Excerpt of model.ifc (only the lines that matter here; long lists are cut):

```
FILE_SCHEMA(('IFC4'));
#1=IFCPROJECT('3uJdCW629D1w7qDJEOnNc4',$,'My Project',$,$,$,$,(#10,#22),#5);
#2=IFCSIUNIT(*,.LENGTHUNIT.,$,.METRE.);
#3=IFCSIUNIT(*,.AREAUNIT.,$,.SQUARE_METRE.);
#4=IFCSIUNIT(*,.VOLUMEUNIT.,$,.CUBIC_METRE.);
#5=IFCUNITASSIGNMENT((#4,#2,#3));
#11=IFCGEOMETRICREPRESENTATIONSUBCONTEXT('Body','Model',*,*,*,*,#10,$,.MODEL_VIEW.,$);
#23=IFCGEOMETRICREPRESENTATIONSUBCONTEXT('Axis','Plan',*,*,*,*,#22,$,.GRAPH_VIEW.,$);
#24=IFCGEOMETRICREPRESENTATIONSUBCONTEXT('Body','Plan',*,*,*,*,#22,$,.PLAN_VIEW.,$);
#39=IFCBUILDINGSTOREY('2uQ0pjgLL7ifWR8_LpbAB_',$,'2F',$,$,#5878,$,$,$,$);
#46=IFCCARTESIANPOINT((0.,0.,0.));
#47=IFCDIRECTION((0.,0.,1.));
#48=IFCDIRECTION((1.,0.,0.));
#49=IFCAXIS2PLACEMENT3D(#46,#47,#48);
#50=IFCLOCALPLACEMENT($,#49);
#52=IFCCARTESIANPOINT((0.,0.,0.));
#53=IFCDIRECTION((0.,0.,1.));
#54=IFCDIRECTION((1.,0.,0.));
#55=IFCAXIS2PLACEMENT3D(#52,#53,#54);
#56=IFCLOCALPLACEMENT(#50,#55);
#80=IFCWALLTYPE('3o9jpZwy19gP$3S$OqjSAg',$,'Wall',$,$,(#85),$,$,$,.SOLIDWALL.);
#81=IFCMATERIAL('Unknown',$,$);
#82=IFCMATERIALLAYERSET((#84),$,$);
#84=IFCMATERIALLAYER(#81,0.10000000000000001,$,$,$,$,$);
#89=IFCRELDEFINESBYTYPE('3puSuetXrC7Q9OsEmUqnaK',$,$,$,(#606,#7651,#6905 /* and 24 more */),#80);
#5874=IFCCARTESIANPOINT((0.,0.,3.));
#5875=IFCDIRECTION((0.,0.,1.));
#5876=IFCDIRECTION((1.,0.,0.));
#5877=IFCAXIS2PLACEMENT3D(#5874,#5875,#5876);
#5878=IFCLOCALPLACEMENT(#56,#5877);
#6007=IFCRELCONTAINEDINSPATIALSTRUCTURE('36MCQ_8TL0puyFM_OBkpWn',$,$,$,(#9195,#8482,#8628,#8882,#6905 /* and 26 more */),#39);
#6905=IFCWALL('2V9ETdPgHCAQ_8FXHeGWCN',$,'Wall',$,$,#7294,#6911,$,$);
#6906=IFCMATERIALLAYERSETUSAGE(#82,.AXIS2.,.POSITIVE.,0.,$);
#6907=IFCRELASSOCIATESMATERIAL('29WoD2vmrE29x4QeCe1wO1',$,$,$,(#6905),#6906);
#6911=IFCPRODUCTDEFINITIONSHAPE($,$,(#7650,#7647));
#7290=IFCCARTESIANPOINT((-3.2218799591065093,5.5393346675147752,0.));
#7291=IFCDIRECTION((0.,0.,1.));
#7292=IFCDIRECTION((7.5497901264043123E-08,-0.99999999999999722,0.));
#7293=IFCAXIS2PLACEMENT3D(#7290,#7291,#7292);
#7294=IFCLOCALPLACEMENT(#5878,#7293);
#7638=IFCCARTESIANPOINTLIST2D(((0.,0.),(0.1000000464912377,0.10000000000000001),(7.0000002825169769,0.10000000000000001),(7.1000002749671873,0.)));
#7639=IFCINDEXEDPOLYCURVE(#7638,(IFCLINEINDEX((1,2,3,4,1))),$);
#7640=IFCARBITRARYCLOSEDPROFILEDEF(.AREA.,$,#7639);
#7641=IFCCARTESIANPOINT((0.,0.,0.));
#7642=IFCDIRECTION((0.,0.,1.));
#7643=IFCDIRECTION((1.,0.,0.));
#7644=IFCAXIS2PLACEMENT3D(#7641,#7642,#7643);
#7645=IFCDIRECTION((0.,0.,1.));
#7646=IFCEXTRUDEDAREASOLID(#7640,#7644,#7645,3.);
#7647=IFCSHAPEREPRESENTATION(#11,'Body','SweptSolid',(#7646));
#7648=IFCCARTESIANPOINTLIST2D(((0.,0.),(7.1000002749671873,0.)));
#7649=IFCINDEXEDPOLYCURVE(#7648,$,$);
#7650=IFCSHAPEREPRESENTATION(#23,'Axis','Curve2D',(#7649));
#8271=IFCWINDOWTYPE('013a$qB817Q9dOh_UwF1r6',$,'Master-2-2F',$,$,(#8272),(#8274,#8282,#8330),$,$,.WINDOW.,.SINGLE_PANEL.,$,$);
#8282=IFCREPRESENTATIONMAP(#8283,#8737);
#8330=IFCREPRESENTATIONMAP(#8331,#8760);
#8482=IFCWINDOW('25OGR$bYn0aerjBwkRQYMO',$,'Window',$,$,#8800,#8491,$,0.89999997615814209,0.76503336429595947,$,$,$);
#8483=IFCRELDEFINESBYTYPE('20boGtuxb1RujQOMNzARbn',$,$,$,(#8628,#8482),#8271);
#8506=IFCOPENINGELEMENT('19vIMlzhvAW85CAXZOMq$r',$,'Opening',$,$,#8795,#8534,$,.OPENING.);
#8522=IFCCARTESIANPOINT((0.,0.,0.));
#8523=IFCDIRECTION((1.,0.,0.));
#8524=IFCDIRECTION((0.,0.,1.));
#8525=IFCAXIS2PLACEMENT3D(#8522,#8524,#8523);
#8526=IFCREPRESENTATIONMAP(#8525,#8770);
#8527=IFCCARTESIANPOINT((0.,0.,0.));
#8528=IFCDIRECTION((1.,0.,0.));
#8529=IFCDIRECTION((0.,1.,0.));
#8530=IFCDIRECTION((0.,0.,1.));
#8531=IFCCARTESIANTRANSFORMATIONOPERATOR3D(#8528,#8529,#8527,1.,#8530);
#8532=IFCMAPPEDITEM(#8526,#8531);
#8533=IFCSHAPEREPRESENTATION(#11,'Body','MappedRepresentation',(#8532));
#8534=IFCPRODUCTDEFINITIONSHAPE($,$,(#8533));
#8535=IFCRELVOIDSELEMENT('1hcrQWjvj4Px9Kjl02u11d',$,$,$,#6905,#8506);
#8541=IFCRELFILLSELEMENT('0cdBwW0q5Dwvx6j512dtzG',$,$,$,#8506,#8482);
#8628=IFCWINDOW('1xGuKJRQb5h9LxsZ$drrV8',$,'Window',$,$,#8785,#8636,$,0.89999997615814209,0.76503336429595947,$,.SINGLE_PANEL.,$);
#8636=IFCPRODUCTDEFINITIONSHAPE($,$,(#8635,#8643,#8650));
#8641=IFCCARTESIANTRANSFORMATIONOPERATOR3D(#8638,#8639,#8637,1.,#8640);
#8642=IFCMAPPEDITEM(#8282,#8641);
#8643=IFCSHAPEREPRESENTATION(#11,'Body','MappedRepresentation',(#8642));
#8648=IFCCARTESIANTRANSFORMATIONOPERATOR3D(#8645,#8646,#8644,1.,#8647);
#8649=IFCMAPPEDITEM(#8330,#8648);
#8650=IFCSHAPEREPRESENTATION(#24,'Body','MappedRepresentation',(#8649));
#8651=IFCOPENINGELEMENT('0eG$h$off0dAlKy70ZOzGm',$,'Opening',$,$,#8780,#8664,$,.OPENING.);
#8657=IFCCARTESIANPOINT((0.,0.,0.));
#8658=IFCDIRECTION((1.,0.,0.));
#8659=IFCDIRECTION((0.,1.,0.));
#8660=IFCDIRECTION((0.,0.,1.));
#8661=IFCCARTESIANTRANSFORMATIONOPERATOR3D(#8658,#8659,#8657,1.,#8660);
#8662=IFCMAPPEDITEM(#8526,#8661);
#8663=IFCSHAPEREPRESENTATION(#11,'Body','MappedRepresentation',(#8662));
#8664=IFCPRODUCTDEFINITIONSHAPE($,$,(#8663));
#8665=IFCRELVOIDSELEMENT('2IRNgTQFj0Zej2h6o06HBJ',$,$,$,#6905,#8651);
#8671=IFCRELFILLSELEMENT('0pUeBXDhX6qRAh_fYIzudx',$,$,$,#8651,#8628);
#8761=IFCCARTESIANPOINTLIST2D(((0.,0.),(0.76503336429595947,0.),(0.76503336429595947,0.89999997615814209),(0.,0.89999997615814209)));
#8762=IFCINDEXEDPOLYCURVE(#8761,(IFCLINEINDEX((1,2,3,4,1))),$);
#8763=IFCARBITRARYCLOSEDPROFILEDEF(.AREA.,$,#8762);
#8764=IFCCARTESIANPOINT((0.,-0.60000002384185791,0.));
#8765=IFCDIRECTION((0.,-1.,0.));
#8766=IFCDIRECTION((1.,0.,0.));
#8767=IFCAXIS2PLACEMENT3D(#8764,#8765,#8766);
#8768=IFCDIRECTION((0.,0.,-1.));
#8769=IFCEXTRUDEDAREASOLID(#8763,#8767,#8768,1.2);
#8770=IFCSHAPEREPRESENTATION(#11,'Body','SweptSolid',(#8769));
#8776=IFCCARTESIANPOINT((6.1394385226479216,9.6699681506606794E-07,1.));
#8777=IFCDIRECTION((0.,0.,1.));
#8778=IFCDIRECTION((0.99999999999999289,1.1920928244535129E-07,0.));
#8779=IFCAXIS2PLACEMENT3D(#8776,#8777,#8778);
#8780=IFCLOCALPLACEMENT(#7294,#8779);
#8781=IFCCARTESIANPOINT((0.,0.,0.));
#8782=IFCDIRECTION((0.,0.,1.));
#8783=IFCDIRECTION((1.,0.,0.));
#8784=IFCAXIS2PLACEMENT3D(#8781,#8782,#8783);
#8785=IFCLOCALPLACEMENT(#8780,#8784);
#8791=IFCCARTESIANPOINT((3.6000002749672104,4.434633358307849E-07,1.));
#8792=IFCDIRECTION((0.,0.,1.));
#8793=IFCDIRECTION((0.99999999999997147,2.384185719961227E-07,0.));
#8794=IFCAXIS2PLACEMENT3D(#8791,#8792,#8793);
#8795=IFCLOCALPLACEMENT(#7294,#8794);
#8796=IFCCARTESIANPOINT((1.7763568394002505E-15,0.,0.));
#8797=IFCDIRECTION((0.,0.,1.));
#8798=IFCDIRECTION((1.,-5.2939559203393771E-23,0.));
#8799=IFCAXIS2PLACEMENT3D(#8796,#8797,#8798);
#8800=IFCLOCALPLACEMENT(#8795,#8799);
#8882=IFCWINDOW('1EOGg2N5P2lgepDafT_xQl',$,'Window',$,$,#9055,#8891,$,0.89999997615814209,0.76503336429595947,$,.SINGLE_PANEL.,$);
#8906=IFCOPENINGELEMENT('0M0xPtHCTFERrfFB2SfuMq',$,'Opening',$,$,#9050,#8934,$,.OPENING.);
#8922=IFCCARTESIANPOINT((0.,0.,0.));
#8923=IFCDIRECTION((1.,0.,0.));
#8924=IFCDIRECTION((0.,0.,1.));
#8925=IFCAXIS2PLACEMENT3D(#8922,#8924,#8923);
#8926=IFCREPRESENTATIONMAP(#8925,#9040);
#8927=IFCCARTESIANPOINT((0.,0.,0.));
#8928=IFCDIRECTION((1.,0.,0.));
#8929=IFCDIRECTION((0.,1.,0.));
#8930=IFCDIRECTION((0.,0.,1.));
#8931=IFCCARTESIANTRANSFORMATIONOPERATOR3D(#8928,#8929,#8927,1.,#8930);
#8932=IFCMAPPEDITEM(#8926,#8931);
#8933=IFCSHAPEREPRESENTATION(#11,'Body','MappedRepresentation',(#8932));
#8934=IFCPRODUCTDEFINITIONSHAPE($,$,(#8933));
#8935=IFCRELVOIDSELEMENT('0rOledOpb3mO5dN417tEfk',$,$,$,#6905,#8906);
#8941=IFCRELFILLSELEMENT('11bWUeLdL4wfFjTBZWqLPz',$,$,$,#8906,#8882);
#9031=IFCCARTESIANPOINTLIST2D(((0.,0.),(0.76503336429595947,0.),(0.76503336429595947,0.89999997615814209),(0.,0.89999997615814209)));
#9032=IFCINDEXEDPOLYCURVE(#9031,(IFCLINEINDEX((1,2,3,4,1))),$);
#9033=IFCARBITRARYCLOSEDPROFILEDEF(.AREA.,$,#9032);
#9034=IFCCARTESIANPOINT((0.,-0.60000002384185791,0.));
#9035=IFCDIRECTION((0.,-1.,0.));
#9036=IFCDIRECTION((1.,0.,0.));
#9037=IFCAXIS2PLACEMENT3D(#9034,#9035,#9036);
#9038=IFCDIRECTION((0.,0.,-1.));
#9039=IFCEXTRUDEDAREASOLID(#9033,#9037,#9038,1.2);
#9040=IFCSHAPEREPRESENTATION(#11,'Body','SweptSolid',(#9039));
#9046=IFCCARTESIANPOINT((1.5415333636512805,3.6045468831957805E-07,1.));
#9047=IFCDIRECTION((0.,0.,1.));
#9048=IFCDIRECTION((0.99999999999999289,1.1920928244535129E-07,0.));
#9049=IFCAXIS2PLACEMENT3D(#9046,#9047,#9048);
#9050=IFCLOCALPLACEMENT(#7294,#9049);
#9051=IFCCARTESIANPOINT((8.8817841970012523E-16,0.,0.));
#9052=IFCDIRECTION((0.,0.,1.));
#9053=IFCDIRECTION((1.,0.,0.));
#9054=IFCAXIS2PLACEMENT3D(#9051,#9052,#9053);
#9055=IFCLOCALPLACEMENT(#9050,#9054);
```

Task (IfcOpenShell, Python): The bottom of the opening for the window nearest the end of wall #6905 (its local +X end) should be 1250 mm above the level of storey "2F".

```python
import numpy as np
import ifcopenshell
import ifcopenshell.api.geometry
import ifcopenshell.geom
import ifcopenshell.util.element
import ifcopenshell.util.placement
import ifcopenshell.util.shape
import ifcopenshell.util.unit

model = ifcopenshell.open("model.ifc")
unit_scale = ifcopenshell.util.unit.calculate_unit_scale(model)

window = model.by_id(8628)
opening = window.FillsVoids[0].RelatingOpeningElement
storey = ifcopenshell.util.element.get_container(window, ifc_class="IfcBuildingStorey")
level = ifcopenshell.util.placement.get_local_placement(storey.ObjectPlacement)[2, 3]

# The opening's origin need not be at the sill, so measure its lowest point.
shape = ifcopenshell.geom.create_shape(ifcopenshell.geom.settings(), opening)
bottom = ifcopenshell.util.shape.get_shape_bottom_elevation(shape, shape.geometry) / unit_scale
dz = level + 1.25 / unit_scale - bottom

shift = np.array([0.0, 0.0, dz])
# The window is placed relative to its opening, so it follows when the opening moves.
matrix = ifcopenshell.util.placement.get_local_placement(opening.ObjectPlacement)
matrix[:3, 3] += shift
ifcopenshell.api.geometry.edit_object_placement(
    model, product=opening, matrix=matrix, is_si=False, should_transform_children=True
)

print(f"moved by {dz * unit_scale:+.3f} m")

model.write("model_edited.ifc")
```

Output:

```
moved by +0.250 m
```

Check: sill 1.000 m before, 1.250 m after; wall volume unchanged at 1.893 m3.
